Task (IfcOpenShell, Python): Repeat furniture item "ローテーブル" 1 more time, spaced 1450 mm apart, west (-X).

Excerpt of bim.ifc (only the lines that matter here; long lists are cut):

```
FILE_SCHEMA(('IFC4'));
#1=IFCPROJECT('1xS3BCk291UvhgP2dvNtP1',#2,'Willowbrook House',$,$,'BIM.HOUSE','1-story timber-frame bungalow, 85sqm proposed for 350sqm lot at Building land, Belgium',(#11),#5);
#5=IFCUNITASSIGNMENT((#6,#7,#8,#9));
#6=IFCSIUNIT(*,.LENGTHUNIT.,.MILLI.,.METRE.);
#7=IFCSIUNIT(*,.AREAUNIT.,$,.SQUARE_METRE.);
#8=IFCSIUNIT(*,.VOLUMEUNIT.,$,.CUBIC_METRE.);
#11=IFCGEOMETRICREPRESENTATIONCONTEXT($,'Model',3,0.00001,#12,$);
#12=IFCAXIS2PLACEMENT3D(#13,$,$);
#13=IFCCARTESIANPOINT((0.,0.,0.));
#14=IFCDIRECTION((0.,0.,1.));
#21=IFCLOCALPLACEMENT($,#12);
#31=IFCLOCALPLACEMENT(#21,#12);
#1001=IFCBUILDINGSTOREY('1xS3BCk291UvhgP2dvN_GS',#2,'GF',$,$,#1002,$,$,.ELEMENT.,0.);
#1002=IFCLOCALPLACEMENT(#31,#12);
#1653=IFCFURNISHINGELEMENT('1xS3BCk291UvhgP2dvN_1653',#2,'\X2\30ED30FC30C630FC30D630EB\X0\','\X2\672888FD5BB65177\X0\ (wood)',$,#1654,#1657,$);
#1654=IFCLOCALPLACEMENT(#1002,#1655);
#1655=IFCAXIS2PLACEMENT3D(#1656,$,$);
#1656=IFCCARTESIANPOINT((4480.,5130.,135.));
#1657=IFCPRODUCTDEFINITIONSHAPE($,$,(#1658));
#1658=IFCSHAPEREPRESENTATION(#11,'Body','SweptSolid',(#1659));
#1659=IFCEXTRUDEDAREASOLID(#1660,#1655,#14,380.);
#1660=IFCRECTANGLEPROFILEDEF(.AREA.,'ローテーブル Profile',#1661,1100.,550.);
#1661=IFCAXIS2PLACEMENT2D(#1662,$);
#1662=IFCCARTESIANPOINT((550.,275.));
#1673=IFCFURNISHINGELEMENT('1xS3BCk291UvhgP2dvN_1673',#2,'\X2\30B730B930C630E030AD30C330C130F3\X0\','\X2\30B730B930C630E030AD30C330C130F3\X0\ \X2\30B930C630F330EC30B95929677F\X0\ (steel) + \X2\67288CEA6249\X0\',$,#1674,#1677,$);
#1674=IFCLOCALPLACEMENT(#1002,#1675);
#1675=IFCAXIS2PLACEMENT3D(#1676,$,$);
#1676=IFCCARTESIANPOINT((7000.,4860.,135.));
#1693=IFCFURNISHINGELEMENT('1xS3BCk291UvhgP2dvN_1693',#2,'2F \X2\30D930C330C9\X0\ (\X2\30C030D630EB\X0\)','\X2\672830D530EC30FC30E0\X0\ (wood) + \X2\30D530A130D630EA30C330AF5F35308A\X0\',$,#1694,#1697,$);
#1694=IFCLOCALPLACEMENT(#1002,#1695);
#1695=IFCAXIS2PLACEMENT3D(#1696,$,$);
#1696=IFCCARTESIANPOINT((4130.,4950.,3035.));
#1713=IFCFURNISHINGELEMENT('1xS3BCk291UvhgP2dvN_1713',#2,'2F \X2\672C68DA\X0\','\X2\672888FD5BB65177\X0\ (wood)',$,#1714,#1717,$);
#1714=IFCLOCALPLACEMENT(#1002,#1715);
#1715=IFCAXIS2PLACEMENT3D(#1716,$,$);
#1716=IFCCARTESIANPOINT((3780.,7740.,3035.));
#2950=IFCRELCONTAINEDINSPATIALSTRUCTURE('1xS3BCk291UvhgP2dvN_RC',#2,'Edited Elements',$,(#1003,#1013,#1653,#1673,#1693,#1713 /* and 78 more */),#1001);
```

```python
import numpy as np
import ifcopenshell
import ifcopenshell.api.geometry
import ifcopenshell.api.root
import ifcopenshell.util.element
import ifcopenshell.util.placement
import ifcopenshell.util.unit

model = ifcopenshell.open("bim.ifc")
unit_scale = ifcopenshell.util.unit.calculate_unit_scale(model)


def reuse_history(source, copy):
    """copy_class also copies each property set's owner history, people and application; keep the originals."""
    for rel in copy.IsDefinedBy:
        if rel.is_a("IfcRelDefinesByProperties") and (history := rel.RelatingPropertyDefinition.OwnerHistory):
            rel.RelatingPropertyDefinition.OwnerHistory = source.OwnerHistory
            ifcopenshell.util.element.remove_deep2(model, history)


source = model.by_id(1653)
base = ifcopenshell.util.placement.get_local_placement(source.ObjectPlacement)
step = np.array([-1.0, 0.0, 0.0]) * 1.45 / unit_scale

for i in range(1, 2):
    copy = ifcopenshell.api.root.copy_class(model, product=source)
    copy.Representation = ifcopenshell.util.element.copy_deep(
        model, source.Representation, exclude=["IfcGeometricRepresentationContext", "IfcRepresentationMap"]
    )
    reuse_history(source, copy)
    matrix = base.copy()
    matrix[:3, 3] += i * step
    print("added at", matrix[:3, 3].round(3) + 0.0)
    ifcopenshell.api.geometry.edit_object_placement(model, product=copy, matrix=matrix, is_si=False)

model.write("bim_rev.ifc")
```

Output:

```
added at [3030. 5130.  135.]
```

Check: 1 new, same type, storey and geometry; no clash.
